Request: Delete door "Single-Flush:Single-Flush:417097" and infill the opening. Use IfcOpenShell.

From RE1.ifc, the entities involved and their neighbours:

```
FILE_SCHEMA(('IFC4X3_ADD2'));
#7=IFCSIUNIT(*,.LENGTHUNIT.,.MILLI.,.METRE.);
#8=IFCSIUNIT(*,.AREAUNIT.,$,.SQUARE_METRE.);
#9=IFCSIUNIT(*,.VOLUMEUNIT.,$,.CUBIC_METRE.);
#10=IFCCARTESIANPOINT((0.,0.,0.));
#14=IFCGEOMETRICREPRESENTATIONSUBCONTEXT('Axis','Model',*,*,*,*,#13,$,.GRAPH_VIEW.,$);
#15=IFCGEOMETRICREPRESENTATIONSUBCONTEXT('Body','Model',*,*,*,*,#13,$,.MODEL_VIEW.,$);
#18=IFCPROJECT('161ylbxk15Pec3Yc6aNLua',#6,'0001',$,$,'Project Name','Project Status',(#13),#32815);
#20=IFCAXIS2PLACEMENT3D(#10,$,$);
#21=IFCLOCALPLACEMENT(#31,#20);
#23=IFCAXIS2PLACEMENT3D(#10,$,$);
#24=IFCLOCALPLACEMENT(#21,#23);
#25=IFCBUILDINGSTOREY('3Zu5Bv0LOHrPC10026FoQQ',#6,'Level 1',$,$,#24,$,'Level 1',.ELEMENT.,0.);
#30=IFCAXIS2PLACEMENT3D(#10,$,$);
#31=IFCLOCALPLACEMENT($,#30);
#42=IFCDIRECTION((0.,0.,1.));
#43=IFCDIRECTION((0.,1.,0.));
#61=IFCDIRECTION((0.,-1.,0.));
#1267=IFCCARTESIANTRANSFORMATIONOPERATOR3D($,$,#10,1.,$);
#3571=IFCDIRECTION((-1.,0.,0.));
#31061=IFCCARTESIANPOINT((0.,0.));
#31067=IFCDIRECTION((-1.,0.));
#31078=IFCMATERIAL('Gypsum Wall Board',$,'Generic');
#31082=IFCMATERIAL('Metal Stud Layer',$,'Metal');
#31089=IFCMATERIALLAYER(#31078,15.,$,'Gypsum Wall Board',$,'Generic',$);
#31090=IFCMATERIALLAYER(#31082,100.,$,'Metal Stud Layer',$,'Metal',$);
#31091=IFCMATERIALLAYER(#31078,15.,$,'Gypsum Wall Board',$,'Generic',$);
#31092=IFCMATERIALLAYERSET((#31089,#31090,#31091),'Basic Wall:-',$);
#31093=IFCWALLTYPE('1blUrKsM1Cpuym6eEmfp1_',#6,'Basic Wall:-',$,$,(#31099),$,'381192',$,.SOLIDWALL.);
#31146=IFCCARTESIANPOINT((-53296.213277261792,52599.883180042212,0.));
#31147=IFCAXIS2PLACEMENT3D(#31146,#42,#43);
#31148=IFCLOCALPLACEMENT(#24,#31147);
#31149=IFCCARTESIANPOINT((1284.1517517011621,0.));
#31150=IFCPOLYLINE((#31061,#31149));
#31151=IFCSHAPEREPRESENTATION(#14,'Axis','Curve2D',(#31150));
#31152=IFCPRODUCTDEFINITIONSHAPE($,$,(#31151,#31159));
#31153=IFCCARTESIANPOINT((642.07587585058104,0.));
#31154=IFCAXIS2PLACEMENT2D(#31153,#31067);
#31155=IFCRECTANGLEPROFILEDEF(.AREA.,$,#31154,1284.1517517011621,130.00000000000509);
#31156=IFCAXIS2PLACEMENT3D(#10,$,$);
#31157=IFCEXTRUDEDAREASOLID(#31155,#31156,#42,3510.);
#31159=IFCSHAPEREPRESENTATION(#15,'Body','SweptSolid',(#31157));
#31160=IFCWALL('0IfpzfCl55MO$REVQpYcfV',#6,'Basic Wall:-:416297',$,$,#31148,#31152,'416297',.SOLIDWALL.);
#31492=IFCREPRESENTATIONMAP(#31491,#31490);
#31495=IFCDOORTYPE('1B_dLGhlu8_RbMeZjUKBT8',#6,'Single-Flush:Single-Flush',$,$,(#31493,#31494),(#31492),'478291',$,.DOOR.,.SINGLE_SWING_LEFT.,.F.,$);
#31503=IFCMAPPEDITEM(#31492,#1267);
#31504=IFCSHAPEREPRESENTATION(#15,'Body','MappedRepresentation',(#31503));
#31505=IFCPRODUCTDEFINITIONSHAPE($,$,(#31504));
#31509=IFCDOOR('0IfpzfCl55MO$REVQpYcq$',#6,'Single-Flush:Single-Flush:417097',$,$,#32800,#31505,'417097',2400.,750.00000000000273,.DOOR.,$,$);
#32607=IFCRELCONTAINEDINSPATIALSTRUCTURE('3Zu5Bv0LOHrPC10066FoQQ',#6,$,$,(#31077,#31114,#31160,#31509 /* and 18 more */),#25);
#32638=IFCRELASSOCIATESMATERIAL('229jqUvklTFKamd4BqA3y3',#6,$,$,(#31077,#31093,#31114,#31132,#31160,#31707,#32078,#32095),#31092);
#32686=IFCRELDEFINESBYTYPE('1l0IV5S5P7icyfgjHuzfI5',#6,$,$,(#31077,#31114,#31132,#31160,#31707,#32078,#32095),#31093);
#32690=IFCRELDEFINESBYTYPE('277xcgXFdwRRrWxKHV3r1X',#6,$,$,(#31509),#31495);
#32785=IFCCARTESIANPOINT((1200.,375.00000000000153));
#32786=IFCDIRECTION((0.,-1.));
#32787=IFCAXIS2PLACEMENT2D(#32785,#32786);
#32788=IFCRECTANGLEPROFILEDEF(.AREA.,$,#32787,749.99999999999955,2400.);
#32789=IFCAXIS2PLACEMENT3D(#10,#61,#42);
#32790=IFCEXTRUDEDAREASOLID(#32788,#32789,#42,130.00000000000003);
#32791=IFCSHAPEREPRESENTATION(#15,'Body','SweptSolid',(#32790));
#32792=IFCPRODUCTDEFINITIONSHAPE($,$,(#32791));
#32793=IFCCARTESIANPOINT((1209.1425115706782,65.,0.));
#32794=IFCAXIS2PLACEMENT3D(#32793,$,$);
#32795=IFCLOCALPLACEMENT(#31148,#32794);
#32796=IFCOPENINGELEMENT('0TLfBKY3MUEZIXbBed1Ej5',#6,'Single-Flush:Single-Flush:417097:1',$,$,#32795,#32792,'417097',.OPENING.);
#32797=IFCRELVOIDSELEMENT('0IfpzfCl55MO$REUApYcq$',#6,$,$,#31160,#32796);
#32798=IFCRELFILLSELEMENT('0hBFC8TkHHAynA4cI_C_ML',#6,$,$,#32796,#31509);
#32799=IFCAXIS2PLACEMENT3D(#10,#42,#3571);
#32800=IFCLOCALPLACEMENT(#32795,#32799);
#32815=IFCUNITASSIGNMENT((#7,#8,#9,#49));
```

```python
import ifcopenshell
import ifcopenshell.api.feature
import ifcopenshell.api.root
import ifcopenshell.geom
import ifcopenshell.util.shape

model = ifcopenshell.open("RE1.ifc")
settings = ifcopenshell.geom.settings()


def volume(element):
    """Net volume in cubic metres, openings subtracted."""
    shape = ifcopenshell.geom.create_shape(settings, element)
    return ifcopenshell.util.shape.get_volume(shape.geometry)


door = model.by_guid("0IfpzfCl55MO$REVQpYcq$")
opening = door.FillsVoids[0].RelatingOpeningElement
wall = opening.VoidsElements[0].RelatingBuildingElement
before = volume(wall)

ifcopenshell.api.root.remove_product(model, product=door)
ifcopenshell.api.feature.remove_feature(model, feature=opening)

after = volume(wall)

print(f"wall volume {before:.3f} -> {after:.3f} m3")

model.write("RE1_v2.ifc")
```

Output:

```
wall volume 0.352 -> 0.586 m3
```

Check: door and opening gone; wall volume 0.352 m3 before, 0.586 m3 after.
